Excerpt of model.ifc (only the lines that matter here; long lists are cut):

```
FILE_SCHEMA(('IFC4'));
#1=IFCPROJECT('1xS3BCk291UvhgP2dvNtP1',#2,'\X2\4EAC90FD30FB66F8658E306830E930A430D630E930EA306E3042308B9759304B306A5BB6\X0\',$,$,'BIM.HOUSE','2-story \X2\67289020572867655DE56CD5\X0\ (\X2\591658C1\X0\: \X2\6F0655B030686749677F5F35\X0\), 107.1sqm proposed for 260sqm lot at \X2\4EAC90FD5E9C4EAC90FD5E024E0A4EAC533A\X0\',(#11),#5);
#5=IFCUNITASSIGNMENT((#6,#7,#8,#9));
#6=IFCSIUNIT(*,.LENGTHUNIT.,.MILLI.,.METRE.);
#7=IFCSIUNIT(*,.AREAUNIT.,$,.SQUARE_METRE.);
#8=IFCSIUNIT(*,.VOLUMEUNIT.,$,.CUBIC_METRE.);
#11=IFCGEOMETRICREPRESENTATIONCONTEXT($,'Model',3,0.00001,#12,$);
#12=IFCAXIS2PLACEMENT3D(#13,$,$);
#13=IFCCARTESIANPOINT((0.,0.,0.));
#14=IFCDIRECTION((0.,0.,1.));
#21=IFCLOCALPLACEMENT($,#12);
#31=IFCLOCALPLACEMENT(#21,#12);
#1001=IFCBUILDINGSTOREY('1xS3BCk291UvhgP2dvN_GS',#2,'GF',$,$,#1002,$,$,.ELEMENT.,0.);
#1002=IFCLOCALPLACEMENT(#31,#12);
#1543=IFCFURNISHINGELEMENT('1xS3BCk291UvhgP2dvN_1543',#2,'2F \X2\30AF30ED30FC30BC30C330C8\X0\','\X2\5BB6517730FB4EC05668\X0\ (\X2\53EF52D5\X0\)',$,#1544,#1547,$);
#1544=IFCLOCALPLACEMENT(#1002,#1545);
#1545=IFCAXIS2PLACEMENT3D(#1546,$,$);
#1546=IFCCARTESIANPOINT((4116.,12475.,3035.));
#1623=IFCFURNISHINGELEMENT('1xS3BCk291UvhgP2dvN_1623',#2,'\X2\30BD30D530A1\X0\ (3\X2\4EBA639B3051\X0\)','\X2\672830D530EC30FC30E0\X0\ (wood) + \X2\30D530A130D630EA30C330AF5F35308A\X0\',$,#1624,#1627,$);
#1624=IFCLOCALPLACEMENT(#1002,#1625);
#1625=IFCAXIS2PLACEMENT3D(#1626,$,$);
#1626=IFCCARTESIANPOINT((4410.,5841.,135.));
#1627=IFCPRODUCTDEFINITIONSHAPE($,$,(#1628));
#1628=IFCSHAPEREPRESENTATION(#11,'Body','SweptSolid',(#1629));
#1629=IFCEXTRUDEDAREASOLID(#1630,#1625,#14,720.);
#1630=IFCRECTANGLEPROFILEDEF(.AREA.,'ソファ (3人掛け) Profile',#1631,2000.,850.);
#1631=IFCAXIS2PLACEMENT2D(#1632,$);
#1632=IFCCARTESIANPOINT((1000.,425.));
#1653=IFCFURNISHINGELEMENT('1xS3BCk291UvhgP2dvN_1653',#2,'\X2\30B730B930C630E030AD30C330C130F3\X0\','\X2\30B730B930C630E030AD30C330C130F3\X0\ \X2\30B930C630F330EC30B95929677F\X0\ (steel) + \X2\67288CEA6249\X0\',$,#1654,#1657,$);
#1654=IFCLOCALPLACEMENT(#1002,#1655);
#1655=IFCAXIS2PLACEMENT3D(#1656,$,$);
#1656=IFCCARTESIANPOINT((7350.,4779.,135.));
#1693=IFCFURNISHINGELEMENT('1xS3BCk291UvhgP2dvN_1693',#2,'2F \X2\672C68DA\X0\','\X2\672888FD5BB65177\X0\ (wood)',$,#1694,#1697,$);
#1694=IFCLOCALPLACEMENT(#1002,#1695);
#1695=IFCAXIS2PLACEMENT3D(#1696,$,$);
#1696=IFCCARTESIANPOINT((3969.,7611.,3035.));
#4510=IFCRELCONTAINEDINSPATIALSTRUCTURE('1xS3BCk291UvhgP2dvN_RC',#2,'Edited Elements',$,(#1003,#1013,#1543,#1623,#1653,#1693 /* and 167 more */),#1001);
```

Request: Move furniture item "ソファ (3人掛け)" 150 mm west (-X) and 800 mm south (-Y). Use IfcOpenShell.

```python
import ifcopenshell
import ifcopenshell.api.geometry
import ifcopenshell.util.placement

model = ifcopenshell.open("model.ifc")

item = model.by_id(1623)
matrix = ifcopenshell.util.placement.get_local_placement(item.ObjectPlacement)
matrix[0, 3] -= 150.0
matrix[1, 3] -= 800.0
ifcopenshell.api.geometry.edit_object_placement(model, product=item, matrix=matrix, is_si=False)

print(ifcopenshell.util.placement.get_local_placement(item.ObjectPlacement).round(3) + 0.0)

model.write("model-out.ifc")
```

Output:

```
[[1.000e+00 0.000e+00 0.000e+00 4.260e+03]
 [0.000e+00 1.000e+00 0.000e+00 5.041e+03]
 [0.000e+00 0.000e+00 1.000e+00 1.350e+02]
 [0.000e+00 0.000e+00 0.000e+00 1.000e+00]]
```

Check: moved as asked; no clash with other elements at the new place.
